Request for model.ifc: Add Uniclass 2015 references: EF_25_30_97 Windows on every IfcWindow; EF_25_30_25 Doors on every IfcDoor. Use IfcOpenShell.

First a look at what the model holds.

```python
import ifcopenshell

model = ifcopenshell.open("model.ifc")
print(model.schema)
print("classifications:", [c.Name for c in model.by_type("IfcClassification")])
for ifc_class in ("IfcDoor", "IfcRoof", "IfcStair", "IfcWall", "IfcWindow"):
    print(ifc_class, len(model.by_type(ifc_class)))
```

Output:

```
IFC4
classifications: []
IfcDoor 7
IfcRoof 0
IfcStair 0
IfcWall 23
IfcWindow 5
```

```python
import ifcopenshell
import ifcopenshell.api.classification

model = ifcopenshell.open("model.ifc")

system = ifcopenshell.api.classification.add_classification(model, classification="Uniclass 2015")

codes = {
    "IfcWindow": ("EF_25_30_97", "Windows"),
    "IfcDoor": ("EF_25_30_25", "Doors"),
}
for ifc_class, (code, name) in codes.items():
    products = model.by_type(ifc_class)
    ifcopenshell.api.classification.add_reference(
        model, products=products, classification=system, identification=code, name=name
    )
    print(code, len(products))

model.write("model_edited.ifc")
```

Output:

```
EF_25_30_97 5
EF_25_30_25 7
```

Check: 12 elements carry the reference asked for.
